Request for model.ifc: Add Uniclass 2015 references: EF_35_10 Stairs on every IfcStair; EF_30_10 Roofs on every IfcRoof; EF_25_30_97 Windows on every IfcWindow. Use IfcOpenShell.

First a look at what the model holds.

```python
import ifcopenshell

model = ifcopenshell.open("model.ifc")
print(model.schema)
print("classifications:", [c.Name for c in model.by_type("IfcClassification")])
for ifc_class in ("IfcDoor", "IfcRoof", "IfcStair", "IfcWall", "IfcWindow"):
    print(ifc_class, len(model.by_type(ifc_class)))
```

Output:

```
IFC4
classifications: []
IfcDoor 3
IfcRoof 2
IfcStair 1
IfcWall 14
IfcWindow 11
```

```python
import ifcopenshell
import ifcopenshell.api.classification

model = ifcopenshell.open("model.ifc")

system = ifcopenshell.api.classification.add_classification(model, classification="Uniclass 2015")

codes = {
    "IfcStair": ("EF_35_10", "Stairs"),
    "IfcRoof": ("EF_30_10", "Roofs"),
    "IfcWindow": ("EF_25_30_97", "Windows"),
}
for ifc_class, (code, name) in codes.items():
    products = model.by_type(ifc_class)
    ifcopenshell.api.classification.add_reference(
        model, products=products, classification=system, identification=code, name=name
    )
    print(code, len(products))

model.write("model_v2.ifc")
```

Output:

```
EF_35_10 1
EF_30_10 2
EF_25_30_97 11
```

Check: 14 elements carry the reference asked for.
